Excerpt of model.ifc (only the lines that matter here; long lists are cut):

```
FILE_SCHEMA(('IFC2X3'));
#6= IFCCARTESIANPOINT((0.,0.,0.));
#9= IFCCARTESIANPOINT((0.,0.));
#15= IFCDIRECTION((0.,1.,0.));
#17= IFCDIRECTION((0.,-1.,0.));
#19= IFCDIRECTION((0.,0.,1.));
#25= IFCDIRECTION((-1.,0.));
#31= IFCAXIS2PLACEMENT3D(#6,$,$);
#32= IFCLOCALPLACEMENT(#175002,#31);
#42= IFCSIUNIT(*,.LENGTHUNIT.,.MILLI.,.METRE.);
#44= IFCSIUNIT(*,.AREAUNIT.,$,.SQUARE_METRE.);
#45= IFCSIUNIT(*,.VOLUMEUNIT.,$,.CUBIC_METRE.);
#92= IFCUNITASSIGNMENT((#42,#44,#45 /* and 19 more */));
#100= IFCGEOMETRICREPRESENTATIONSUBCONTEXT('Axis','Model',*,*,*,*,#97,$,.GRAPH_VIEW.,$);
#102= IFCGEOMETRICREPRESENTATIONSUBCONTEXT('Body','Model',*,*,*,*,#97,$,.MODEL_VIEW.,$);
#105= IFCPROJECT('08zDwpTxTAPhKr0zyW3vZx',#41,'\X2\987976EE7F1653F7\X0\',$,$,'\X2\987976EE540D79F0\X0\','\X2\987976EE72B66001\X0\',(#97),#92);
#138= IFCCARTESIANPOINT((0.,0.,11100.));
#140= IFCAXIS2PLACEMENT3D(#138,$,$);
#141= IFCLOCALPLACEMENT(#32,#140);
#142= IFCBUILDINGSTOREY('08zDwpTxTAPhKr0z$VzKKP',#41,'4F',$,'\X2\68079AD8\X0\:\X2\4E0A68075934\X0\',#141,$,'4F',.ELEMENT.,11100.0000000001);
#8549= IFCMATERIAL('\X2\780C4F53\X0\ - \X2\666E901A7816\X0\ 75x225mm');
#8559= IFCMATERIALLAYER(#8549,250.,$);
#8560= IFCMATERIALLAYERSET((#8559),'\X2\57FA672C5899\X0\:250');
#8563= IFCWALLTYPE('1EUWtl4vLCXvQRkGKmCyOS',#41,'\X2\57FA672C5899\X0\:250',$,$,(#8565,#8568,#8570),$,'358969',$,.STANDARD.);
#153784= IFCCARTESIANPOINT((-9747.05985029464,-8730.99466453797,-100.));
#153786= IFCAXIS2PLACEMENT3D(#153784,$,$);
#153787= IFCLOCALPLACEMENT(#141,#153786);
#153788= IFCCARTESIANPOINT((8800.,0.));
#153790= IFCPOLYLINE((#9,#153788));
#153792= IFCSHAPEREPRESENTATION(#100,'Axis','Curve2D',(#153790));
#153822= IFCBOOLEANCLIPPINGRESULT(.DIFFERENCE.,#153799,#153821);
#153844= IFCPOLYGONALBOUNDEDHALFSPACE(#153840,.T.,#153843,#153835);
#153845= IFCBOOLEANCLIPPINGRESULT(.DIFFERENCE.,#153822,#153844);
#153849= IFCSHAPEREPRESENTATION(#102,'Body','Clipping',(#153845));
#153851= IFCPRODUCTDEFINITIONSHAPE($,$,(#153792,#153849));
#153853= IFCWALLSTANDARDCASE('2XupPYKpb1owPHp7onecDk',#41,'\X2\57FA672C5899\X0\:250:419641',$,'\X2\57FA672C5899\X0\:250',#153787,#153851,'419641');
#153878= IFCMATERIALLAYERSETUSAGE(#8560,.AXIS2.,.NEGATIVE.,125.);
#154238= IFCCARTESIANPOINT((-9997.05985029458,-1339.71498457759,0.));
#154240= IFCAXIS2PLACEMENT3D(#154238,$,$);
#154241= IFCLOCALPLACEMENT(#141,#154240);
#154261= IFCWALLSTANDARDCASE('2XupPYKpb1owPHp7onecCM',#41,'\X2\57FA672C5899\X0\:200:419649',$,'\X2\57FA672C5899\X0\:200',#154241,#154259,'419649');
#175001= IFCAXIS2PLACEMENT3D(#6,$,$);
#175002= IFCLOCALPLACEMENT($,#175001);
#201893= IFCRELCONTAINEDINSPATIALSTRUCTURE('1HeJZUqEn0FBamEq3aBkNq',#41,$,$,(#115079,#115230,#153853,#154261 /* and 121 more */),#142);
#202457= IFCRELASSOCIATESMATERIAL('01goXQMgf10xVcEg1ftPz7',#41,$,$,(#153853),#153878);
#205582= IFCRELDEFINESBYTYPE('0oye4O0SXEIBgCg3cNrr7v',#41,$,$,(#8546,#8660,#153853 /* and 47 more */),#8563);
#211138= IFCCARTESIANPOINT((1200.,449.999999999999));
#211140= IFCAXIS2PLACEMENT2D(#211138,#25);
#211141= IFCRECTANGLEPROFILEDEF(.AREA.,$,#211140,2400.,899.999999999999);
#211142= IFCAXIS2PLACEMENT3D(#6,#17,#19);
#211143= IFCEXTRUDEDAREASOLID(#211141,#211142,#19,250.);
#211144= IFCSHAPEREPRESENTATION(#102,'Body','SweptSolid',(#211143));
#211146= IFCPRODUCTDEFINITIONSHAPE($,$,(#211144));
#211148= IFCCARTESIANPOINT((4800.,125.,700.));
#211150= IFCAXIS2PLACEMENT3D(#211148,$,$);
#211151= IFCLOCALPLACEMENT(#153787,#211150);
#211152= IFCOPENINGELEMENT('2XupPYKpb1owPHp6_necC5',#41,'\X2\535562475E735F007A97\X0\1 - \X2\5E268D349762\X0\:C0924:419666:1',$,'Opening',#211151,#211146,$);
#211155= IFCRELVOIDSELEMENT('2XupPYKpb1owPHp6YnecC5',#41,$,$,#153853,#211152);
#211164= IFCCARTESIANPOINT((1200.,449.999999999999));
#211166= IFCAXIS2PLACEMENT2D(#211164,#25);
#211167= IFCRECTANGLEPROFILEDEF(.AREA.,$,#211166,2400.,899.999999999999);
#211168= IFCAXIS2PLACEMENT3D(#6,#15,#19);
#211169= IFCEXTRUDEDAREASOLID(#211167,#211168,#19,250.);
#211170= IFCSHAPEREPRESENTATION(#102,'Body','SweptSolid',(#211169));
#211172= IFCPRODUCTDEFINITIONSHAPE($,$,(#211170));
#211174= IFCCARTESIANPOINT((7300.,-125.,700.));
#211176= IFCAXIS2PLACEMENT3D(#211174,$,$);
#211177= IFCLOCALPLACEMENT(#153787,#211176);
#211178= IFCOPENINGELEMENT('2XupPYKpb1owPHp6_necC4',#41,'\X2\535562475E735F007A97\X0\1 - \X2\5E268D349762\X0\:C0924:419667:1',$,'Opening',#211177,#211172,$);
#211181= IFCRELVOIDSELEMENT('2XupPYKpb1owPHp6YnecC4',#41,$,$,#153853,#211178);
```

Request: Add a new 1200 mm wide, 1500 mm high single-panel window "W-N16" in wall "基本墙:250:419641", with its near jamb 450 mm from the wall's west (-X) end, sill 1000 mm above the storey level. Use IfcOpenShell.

```python
import numpy as np
import ifcopenshell
import ifcopenshell.api.feature
import ifcopenshell.api.geometry
import ifcopenshell.api.root
import ifcopenshell.api.spatial
import ifcopenshell.api.type
import ifcopenshell.geom
import ifcopenshell.util.element
import ifcopenshell.util.placement
import ifcopenshell.util.representation
import ifcopenshell.util.shape
import ifcopenshell.util.unit

model = ifcopenshell.open("model.ifc")
unit_scale = ifcopenshell.util.unit.calculate_unit_scale(model)
settings = ifcopenshell.geom.settings()


def volume(element):
    """Net volume in cubic metres, openings subtracted."""
    shape = ifcopenshell.geom.create_shape(settings, element)
    return ifcopenshell.util.shape.get_volume(shape.geometry)


wall = model.by_guid("2XupPYKpb1owPHp7onecDk")
storey = ifcopenshell.util.element.get_container(wall, ifc_class="IfcBuildingStorey")
context = ifcopenshell.util.representation.get_context(model, "Model", "Body", "MODEL_VIEW")
before = volume(wall)

width, height, from_end, sill = 1.2, 1.5, 0.45, 1  # metres

# The wall runs along its own X axis, and the end named is its -X end.
wall_shape = ifcopenshell.geom.create_shape(settings, wall)
x, y, z = ifcopenshell.util.shape.get_vertices(wall_shape.geometry).T
start = x.min() + from_end
face, thickness = float(y.min()), float(y.max() - y.min())
wall_matrix = ifcopenshell.util.placement.get_local_placement(wall.ObjectPlacement)
level = ifcopenshell.util.placement.get_local_placement(storey.ObjectPlacement)[2, 3]


def in_wall(x, y):
    """Placement at x, y metres in the wall's axes, at sill height."""
    matrix = wall_matrix.copy()
    matrix[:, 3] = wall_matrix @ np.array([x / unit_scale, y / unit_scale, 0.0, 1.0])
    matrix[2, 3] = level + sill / unit_scale
    return matrix


# Opening: a box that overshoots both wall faces by 50 mm.
opening = ifcopenshell.api.root.create_entity(model, ifc_class="IfcOpeningElement")
box = ifcopenshell.api.geometry.add_wall_representation(
    model, context=context, length=width, height=height, thickness=thickness + 0.1
)
ifcopenshell.api.geometry.assign_representation(model, product=opening, representation=box)
ifcopenshell.api.geometry.edit_object_placement(model, product=opening, matrix=in_wall(start, face - 0.05), is_si=False)
ifcopenshell.api.feature.add_feature(model, feature=opening, element=wall)

window = ifcopenshell.api.root.create_entity(model, ifc_class="IfcWindow", name="W-N16")
window.OverallWidth, window.OverallHeight = width / unit_scale, height / unit_scale
body = ifcopenshell.api.geometry.add_window_representation(
    model,
    context=context,
    overall_width=window.OverallWidth,
    overall_height=window.OverallHeight,
    partition_type="SINGLE_PANEL",
)
ifcopenshell.api.geometry.assign_representation(model, product=window, representation=body)
ifcopenshell.api.spatial.assign_container(model, products=[window], relating_structure=storey)
fills = ifcopenshell.api.feature.add_filling(model, opening=opening, element=window)
fills.OwnerHistory = window.OwnerHistory  # required in IFC2X3

# IFC2X3 keeps the operation on the window style.
style = ifcopenshell.api.root.create_entity(model, ifc_class="IfcWindowStyle", name="W-N16")
style.OperationType, style.ConstructionType = "SINGLE_PANEL", "NOTDEFINED"
style.ParameterTakesPrecedence = style.Sizeable = False
ifcopenshell.api.type.assign_type(model, related_objects=[window], relating_type=style)

# Centre the window in the wall's thickness.
ifcopenshell.api.geometry.edit_object_placement(model, product=window, matrix=in_wall(start, face), is_si=False)
window_shape = ifcopenshell.geom.create_shape(settings, window)
depth = ifcopenshell.util.shape.get_vertices(window_shape.geometry)[:, 1]
offset = face + thickness / 2 - (depth.min() + depth.max()) / 2
ifcopenshell.api.geometry.edit_object_placement(model, product=window, matrix=in_wall(start, offset), is_si=False)

after = volume(wall)

print(f"wall volume {before:.3f} -> {after:.3f} m3")

model.write("model_v2.ifc")
```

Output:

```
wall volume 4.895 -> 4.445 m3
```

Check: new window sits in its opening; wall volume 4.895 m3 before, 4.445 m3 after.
